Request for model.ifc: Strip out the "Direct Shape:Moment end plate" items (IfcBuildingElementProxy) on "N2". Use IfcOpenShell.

First a look at what the model holds.

```python
import ifcopenshell
import ifcopenshell.util.element

model = ifcopenshell.open("model.ifc")
print(model.schema)
storey = next(s for s in model.by_type("IfcBuildingStorey") if s.Name == "N2")
proxies = [e for e in ifcopenshell.util.element.get_decomposition(storey) if e.is_a("IfcBuildingElementProxy")]
seen = {}
for e in proxies:
    element_type = ifcopenshell.util.element.get_type(e)
    name = element_type.Name if element_type not in (None, e) else None
    seen[name] = seen.get(name, 0) + 1
for name, count in sorted(seen.items(), key=str):
    print(count, "x", name)
```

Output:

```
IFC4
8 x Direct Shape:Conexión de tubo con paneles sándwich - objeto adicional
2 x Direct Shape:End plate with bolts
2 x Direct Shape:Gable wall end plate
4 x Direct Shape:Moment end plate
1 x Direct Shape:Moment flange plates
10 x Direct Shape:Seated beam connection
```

```python
import ifcopenshell
import ifcopenshell.api.root
import ifcopenshell.util.element

model = ifcopenshell.open("model.ifc")

storey = next(s for s in model.by_type("IfcBuildingStorey") if s.Name == "N2")
proxies = [e for e in ifcopenshell.util.element.get_decomposition(storey) if e.is_a("IfcBuildingElementProxy")]
targets = [e for e in proxies if (t := ifcopenshell.util.element.get_type(e)) not in (None, e) and t.Name == "Direct Shape:Moment end plate"]

for e in targets:
    ifcopenshell.api.root.remove_product(model, product=e)
print(len(targets), "removed")

model.write("model_edited.ifc")
```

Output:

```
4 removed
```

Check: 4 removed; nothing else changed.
